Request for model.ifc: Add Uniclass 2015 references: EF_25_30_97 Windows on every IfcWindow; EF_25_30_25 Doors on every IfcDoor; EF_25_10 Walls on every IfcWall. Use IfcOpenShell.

First a look at what the model holds.

```python
import ifcopenshell

model = ifcopenshell.open("model.ifc")
print(model.schema)
print("classifications:", [c.Name for c in model.by_type("IfcClassification")])
for ifc_class in ("IfcDoor", "IfcRoof", "IfcStair", "IfcWall", "IfcWindow"):
    print(ifc_class, len(model.by_type(ifc_class)))
```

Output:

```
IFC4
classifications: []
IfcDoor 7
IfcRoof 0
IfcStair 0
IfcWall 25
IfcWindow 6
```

```python
import ifcopenshell
import ifcopenshell.api.classification

model = ifcopenshell.open("model.ifc")

system = ifcopenshell.api.classification.add_classification(model, classification="Uniclass 2015")

codes = {
    "IfcWindow": ("EF_25_30_97", "Windows"),
    "IfcDoor": ("EF_25_30_25", "Doors"),
    "IfcWall": ("EF_25_10", "Walls"),
}
for ifc_class, (code, name) in codes.items():
    products = model.by_type(ifc_class)
    ifcopenshell.api.classification.add_reference(
        model, products=products, classification=system, identification=code, name=name
    )
    print(code, len(products))

model.write("model_v2.ifc")
```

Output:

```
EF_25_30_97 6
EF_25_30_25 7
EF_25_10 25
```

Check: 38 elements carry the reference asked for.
